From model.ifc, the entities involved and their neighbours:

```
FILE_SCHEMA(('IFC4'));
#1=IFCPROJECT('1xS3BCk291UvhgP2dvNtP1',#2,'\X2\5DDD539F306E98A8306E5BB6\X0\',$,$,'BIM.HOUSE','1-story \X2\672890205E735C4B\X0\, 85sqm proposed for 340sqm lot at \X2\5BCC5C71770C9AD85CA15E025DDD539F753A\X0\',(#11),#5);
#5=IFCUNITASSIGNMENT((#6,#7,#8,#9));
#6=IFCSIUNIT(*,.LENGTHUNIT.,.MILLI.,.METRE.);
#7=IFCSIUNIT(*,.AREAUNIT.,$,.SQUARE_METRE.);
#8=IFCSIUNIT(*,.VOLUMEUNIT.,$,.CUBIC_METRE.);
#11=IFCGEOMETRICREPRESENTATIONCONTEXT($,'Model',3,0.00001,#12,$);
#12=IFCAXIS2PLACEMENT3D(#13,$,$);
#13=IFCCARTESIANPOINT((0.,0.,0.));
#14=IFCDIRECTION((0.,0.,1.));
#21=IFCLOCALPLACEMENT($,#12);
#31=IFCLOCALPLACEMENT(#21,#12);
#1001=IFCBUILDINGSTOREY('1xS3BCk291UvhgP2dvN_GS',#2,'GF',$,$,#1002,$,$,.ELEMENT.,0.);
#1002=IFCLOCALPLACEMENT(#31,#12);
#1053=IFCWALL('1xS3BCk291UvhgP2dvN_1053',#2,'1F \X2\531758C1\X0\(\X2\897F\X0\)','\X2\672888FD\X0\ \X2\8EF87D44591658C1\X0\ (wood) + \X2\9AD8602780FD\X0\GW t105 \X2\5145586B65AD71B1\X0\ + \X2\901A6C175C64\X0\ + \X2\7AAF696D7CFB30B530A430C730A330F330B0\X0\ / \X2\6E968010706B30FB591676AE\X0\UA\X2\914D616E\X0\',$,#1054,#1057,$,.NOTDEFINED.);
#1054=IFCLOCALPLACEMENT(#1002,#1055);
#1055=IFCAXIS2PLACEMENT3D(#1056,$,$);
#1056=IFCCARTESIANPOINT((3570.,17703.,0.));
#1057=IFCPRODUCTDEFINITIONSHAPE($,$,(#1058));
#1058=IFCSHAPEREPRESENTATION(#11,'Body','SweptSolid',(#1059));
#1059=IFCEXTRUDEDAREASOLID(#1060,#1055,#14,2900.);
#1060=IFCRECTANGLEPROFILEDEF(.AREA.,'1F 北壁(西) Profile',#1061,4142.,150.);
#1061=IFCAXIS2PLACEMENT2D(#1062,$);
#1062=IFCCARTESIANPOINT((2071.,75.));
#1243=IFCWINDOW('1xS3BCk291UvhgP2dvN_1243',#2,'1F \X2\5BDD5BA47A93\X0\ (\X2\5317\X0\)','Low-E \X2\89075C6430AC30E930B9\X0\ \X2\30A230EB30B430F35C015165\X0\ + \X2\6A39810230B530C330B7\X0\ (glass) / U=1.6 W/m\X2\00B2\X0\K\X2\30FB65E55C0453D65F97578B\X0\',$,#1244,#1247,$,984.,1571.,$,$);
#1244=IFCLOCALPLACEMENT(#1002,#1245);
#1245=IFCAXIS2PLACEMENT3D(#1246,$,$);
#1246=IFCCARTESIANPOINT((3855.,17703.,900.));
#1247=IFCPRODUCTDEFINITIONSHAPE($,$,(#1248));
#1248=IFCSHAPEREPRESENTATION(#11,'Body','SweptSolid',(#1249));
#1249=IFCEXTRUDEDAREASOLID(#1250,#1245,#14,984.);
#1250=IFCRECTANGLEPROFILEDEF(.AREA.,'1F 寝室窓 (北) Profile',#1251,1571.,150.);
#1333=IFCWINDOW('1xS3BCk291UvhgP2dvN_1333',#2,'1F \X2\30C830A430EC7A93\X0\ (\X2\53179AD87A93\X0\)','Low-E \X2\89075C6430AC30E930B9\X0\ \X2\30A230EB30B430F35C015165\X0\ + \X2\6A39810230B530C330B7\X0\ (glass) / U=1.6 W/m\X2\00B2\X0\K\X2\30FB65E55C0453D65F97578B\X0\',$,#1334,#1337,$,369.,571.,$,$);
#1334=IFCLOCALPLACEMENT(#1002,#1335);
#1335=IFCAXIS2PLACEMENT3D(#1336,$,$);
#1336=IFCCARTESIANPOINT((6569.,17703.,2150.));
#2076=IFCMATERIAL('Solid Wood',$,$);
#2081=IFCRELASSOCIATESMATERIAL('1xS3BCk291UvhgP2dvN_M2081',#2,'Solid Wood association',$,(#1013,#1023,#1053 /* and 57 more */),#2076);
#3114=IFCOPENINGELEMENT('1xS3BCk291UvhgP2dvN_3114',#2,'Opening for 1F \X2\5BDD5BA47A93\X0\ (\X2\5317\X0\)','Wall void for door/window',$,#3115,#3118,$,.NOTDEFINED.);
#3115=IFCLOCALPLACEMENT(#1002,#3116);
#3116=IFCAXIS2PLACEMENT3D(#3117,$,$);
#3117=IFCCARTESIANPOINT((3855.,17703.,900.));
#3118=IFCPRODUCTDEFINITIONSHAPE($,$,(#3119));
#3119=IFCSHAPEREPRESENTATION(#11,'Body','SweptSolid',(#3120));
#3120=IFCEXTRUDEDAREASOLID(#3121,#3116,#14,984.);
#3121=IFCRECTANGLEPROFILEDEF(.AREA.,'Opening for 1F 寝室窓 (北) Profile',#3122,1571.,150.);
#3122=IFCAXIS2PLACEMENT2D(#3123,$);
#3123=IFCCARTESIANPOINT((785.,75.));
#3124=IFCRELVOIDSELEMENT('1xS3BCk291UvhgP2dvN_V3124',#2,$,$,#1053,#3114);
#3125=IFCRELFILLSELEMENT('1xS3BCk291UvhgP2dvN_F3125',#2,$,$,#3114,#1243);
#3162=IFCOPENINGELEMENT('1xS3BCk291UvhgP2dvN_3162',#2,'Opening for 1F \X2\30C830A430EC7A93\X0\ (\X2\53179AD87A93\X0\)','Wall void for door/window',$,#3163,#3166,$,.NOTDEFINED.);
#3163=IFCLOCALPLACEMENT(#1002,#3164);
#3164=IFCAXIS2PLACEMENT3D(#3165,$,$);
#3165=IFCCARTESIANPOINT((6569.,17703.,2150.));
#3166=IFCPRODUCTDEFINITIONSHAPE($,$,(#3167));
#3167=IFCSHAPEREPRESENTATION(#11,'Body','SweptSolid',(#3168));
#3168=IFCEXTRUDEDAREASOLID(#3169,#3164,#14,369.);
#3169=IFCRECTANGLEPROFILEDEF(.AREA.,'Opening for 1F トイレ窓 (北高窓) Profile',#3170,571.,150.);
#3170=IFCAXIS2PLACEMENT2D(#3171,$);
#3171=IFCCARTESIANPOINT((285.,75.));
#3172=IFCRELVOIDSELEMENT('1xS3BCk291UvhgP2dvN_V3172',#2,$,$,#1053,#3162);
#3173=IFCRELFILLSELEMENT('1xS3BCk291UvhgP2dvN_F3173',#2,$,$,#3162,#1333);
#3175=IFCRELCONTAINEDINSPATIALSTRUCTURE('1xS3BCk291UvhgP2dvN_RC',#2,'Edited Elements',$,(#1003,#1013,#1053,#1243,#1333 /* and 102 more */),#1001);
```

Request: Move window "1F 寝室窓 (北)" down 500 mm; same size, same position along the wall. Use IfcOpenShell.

```python
import numpy as np
import ifcopenshell
import ifcopenshell.api.geometry
import ifcopenshell.util.placement
import ifcopenshell.util.unit

model = ifcopenshell.open("model.ifc")
unit_scale = ifcopenshell.util.unit.calculate_unit_scale(model)

window = model.by_id(1243)
opening = window.FillsVoids[0].RelatingOpeningElement
dz = -500.0

shift = np.array([0.0, 0.0, dz])
# The window is not placed relative to its opening, so move both.
for product in (opening, window):
    matrix = ifcopenshell.util.placement.get_local_placement(product.ObjectPlacement)
    matrix[:3, 3] += shift
    ifcopenshell.api.geometry.edit_object_placement(model, product=product, matrix=matrix, is_si=False)

print(f"moved by {dz * unit_scale:+.3f} m")

model.write("model_updated.ifc")
```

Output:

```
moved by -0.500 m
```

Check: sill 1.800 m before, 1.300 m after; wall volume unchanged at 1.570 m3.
